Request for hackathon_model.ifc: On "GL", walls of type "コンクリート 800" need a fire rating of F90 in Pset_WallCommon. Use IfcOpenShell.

First a look at what the model holds.

```python
import ifcopenshell
import ifcopenshell.util.element

model = ifcopenshell.open("hackathon_model.ifc")
print(model.schema)
storey = next(s for s in model.by_type("IfcBuildingStorey") if s.Name == "GL")
walls = [e for e in ifcopenshell.util.element.get_decomposition(storey) if e.is_a("IfcWall")]
seen = {}
for e in walls:
    element_type = ifcopenshell.util.element.get_type(e)
    key = (element_type.Name if element_type != e and element_type else None, ifcopenshell.util.element.get_pset(e, "Pset_WallCommon", "FireRating"))
    seen[key] = seen.get(key, 0) + 1
for (name, value), count in sorted(seen.items(), key=str):
    print(count, "x", name, "|", value)
```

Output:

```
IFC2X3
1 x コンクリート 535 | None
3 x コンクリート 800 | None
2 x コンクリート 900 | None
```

```python
import ifcopenshell
import ifcopenshell.api.pset
import ifcopenshell.util.element

model = ifcopenshell.open("hackathon_model.ifc")

storey = next(s for s in model.by_type("IfcBuildingStorey") if s.Name == "GL")
walls = [e for e in ifcopenshell.util.element.get_decomposition(storey) if e.is_a("IfcWall")]

count = 0
for e in walls:
    element_type = ifcopenshell.util.element.get_type(e)
    if element_type in (None, e) or element_type.Name != "コンクリート 800":
        continue
    # add_pset returns the element's existing set when there is one.
    pset = ifcopenshell.api.pset.add_pset(model, product=e, name="Pset_WallCommon")
    ifcopenshell.api.pset.edit_pset(model, pset=pset, properties={"FireRating": "F90"})
    count += 1

print(count, "walls updated")

model.write("hackathon_model_rev.ifc")
```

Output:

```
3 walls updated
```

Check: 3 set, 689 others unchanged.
